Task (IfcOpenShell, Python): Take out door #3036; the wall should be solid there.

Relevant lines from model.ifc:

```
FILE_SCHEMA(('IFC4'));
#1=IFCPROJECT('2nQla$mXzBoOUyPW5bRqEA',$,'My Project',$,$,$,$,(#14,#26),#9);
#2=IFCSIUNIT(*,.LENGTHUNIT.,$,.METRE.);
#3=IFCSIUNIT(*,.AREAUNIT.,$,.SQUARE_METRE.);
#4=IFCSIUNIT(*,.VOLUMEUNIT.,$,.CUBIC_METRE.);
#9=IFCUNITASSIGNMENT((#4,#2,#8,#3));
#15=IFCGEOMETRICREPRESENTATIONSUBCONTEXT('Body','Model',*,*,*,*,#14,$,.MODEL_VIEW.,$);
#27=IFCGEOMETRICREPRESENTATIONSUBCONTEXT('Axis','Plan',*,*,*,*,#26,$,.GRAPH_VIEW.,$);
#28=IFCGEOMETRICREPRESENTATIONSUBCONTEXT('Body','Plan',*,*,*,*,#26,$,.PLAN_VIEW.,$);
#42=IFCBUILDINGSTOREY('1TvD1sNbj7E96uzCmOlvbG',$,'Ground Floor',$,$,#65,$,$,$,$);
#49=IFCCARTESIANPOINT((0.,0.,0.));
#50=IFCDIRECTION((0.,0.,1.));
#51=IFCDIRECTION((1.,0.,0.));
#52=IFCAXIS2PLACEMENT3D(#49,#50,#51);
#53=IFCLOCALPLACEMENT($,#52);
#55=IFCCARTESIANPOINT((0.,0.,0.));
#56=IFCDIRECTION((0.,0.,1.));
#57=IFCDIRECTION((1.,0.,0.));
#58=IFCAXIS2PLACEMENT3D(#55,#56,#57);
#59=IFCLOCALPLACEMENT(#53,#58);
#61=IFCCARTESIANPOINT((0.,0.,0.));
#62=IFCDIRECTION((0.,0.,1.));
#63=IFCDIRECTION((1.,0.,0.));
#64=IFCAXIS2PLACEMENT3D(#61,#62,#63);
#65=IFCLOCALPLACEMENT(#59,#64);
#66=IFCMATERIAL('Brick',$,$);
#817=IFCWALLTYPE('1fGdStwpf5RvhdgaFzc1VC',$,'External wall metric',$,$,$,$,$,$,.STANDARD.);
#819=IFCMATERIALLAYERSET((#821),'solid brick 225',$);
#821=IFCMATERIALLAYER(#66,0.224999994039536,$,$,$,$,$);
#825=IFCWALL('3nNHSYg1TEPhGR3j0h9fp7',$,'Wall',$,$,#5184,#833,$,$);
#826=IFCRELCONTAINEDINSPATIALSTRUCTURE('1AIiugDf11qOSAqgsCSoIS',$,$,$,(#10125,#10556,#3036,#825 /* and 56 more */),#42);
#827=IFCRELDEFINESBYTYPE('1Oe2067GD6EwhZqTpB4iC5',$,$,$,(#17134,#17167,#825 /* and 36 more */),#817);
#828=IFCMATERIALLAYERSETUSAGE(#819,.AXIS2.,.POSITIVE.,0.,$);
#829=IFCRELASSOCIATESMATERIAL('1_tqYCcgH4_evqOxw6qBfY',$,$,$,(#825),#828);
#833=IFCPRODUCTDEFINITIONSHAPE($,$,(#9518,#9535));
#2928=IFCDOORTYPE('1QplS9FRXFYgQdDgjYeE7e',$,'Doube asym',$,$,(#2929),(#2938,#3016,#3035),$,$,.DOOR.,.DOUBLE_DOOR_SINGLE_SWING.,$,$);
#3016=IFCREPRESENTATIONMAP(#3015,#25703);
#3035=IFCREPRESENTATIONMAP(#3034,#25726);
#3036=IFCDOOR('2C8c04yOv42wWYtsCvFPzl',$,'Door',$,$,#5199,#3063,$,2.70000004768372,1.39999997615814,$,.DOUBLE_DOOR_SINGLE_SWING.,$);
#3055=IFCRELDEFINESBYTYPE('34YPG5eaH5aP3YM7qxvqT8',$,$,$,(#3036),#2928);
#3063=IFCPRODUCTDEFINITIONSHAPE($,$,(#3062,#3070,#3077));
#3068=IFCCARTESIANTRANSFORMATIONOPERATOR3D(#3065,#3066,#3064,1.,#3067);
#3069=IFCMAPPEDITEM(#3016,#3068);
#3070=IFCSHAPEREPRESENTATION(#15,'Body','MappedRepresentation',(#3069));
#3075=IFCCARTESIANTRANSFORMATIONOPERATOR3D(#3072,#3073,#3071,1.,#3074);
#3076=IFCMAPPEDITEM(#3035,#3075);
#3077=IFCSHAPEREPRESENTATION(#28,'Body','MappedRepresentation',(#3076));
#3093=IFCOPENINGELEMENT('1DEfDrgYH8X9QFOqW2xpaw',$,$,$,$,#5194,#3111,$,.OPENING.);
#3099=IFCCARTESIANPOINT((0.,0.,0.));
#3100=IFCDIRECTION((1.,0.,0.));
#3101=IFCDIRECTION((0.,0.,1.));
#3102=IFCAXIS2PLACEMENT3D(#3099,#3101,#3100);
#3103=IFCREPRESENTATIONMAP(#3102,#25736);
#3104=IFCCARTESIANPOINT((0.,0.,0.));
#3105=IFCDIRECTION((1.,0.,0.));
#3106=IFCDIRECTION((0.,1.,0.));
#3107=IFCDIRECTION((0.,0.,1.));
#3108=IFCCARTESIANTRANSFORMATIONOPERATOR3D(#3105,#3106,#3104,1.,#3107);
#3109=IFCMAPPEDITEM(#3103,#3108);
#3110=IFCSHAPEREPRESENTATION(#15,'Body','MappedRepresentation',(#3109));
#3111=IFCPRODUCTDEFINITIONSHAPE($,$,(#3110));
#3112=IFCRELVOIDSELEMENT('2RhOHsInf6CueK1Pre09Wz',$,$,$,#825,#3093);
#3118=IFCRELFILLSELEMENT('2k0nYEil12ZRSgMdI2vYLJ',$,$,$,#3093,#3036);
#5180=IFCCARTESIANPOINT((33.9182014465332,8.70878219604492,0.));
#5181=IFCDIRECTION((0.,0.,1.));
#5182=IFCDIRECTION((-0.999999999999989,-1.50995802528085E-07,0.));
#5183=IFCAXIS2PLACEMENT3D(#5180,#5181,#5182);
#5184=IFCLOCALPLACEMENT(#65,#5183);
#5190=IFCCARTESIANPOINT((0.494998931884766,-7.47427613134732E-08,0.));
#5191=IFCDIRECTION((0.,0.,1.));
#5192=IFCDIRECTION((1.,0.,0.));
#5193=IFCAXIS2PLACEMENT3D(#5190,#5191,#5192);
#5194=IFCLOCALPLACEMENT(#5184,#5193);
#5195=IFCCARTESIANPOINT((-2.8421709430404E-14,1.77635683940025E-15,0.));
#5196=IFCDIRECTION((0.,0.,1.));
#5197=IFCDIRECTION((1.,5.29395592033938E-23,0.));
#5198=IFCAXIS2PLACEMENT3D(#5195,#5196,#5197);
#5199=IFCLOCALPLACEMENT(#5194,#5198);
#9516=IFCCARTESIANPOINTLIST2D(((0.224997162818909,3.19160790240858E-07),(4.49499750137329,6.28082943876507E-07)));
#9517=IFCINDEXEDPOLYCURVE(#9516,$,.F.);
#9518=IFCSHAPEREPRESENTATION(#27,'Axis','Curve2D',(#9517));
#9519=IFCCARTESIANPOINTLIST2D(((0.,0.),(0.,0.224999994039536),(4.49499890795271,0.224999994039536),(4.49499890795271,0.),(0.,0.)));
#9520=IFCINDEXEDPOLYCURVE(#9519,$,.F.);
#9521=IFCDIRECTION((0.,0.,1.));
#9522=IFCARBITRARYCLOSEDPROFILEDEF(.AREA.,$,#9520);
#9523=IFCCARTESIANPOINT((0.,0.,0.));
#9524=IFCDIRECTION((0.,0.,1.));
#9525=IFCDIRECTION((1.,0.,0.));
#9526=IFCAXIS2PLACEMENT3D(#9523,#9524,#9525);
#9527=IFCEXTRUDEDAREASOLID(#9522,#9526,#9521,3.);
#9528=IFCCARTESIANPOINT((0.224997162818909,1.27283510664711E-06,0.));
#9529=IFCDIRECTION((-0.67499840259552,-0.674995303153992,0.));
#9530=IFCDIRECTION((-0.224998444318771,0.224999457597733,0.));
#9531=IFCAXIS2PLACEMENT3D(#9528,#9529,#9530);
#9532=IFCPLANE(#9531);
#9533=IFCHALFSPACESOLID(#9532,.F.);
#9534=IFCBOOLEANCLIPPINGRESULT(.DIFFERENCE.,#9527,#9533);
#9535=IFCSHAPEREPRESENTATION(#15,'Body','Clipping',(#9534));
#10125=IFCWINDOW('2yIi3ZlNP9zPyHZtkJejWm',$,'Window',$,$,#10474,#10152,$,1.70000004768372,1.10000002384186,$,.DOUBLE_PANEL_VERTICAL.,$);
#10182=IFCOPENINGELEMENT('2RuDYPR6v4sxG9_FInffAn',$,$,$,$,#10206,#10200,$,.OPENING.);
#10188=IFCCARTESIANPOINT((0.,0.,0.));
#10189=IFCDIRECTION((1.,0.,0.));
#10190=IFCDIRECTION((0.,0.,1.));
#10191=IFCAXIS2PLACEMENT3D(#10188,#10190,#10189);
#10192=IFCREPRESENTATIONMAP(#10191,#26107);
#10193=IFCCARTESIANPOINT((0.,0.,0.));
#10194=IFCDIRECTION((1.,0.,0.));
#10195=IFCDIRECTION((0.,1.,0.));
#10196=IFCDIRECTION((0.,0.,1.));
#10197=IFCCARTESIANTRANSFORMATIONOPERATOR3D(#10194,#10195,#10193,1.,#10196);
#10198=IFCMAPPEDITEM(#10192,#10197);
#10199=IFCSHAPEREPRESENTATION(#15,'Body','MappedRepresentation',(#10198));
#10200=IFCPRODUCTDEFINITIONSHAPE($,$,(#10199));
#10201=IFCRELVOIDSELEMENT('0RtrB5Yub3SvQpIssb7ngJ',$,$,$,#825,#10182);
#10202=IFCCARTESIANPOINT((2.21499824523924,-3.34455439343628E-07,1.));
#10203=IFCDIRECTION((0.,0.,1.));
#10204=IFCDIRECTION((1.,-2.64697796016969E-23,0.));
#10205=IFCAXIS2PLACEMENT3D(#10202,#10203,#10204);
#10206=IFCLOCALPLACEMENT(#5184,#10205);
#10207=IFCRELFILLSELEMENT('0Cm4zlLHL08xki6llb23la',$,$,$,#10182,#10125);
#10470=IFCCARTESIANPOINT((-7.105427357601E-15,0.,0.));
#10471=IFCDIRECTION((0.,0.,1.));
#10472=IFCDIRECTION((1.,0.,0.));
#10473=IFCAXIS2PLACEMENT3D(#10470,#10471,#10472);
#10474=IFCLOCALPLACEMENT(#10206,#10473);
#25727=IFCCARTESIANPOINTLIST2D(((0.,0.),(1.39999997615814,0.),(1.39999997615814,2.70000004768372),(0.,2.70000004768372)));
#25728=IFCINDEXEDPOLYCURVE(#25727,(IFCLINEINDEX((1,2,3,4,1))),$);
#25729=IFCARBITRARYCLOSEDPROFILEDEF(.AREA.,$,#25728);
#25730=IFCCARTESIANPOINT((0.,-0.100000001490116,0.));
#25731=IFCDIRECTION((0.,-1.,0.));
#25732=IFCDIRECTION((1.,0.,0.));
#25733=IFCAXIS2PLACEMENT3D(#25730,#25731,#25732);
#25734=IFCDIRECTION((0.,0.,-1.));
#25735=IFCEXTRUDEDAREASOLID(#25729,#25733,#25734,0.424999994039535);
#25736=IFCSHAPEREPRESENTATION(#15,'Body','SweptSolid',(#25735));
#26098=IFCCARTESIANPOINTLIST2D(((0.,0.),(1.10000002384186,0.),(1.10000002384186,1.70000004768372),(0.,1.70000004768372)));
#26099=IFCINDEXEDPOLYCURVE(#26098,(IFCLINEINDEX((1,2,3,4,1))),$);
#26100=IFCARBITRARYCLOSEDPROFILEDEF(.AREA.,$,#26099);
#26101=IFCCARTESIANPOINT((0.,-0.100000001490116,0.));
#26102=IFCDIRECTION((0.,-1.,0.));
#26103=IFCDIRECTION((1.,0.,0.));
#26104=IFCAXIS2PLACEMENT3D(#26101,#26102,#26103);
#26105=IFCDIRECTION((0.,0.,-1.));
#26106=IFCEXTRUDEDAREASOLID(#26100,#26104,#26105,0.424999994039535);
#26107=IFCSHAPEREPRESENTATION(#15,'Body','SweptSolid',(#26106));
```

```python
import ifcopenshell
import ifcopenshell.api.feature
import ifcopenshell.api.root
import ifcopenshell.geom
import ifcopenshell.util.shape

model = ifcopenshell.open("model.ifc")
settings = ifcopenshell.geom.settings()


def volume(element):
    """Net volume in cubic metres, openings subtracted."""
    shape = ifcopenshell.geom.create_shape(settings, element)
    return ifcopenshell.util.shape.get_volume(shape.geometry)


door = model.by_guid("2C8c04yOv42wWYtsCvFPzl")
opening = door.FillsVoids[0].RelatingOpeningElement
wall = opening.VoidsElements[0].RelatingBuildingElement
before = volume(wall)

ifcopenshell.api.root.remove_product(model, product=door)
ifcopenshell.api.feature.remove_feature(model, feature=opening)

after = volume(wall)

print(f"wall volume {before:.3f} -> {after:.3f} m3")

model.write("model-out.ifc")
```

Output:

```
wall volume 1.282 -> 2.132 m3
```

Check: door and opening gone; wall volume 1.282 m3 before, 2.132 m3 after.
